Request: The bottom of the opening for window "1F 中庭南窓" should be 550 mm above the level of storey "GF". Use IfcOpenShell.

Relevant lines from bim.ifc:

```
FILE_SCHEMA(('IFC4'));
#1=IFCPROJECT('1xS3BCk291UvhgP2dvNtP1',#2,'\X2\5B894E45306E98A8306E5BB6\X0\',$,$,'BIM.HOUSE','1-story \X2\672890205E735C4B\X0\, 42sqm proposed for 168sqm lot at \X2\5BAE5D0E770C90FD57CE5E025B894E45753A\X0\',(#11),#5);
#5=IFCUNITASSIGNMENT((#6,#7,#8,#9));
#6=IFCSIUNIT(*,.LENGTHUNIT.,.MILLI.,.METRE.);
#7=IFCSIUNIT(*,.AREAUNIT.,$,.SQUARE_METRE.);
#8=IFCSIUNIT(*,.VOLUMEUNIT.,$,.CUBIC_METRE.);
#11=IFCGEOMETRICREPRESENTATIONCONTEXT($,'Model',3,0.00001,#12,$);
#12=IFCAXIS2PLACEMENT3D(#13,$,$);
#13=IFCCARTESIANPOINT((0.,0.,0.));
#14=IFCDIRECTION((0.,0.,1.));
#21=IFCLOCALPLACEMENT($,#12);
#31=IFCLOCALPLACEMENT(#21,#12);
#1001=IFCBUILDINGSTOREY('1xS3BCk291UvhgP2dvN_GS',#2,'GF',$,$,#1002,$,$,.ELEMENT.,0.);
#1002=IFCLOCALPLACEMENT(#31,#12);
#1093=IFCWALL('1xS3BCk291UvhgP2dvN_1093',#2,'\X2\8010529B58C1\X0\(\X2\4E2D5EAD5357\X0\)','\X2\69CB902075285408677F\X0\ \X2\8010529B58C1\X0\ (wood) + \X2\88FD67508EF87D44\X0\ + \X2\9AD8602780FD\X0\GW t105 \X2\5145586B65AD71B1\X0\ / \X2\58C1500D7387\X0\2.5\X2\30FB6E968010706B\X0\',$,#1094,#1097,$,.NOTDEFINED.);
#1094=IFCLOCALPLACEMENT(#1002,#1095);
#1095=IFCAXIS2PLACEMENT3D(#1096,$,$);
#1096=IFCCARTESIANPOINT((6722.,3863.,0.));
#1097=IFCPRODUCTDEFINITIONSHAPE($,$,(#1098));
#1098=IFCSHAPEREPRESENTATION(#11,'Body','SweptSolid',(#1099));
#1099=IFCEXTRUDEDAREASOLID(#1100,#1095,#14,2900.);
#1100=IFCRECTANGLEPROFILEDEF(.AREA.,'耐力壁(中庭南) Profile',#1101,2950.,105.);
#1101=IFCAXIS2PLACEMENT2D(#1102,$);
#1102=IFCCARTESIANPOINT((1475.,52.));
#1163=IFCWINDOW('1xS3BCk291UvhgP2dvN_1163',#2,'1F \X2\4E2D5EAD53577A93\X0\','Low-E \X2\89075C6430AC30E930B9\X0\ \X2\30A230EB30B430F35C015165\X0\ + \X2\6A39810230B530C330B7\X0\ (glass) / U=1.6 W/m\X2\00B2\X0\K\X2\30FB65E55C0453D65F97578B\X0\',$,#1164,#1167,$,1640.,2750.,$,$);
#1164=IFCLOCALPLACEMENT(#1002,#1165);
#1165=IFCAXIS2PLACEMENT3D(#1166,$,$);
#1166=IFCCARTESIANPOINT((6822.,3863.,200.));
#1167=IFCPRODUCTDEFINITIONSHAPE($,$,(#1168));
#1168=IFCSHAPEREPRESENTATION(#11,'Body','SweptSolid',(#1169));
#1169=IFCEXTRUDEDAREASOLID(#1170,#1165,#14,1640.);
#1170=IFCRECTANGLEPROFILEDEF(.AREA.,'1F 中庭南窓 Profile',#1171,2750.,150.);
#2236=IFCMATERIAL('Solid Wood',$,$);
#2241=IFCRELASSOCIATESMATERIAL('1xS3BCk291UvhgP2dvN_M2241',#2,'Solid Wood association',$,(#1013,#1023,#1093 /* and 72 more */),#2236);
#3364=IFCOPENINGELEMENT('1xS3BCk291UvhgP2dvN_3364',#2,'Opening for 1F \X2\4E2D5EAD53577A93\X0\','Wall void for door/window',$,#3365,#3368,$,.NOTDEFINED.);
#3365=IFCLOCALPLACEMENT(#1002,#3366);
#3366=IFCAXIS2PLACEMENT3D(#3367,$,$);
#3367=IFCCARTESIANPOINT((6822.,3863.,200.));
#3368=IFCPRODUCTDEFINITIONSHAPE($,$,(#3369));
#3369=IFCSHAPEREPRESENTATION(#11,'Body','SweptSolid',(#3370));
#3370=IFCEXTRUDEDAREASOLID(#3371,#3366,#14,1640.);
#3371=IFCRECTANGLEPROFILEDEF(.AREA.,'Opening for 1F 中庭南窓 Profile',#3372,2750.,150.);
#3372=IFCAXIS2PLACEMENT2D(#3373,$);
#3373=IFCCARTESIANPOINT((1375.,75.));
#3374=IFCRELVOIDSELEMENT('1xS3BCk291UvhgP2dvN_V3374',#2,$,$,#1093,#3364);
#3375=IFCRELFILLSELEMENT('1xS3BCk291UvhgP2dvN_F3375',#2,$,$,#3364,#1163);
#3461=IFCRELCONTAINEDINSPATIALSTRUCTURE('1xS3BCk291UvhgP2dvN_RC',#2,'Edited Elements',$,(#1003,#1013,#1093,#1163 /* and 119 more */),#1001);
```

```python
import numpy as np
import ifcopenshell
import ifcopenshell.api.geometry
import ifcopenshell.geom
import ifcopenshell.util.element
import ifcopenshell.util.placement
import ifcopenshell.util.shape
import ifcopenshell.util.unit

model = ifcopenshell.open("bim.ifc")
unit_scale = ifcopenshell.util.unit.calculate_unit_scale(model)

window = model.by_guid("1xS3BCk291UvhgP2dvN_1163")
opening = window.FillsVoids[0].RelatingOpeningElement
storey = ifcopenshell.util.element.get_container(window, ifc_class="IfcBuildingStorey")
level = ifcopenshell.util.placement.get_local_placement(storey.ObjectPlacement)[2, 3]

# The opening's origin need not be at the sill, so measure its lowest point.
shape = ifcopenshell.geom.create_shape(ifcopenshell.geom.settings(), opening)
bottom = ifcopenshell.util.shape.get_shape_bottom_elevation(shape, shape.geometry) / unit_scale
dz = level + 550.0 - bottom

shift = np.array([0.0, 0.0, dz])
# The window is not placed relative to its opening, so move both.
for product in (opening, window):
    matrix = ifcopenshell.util.placement.get_local_placement(product.ObjectPlacement)
    matrix[:3, 3] += shift
    ifcopenshell.api.geometry.edit_object_placement(model, product=product, matrix=matrix, is_si=False)

print(f"moved by {dz * unit_scale:+.3f} m")

model.write("bim_rev.ifc")
```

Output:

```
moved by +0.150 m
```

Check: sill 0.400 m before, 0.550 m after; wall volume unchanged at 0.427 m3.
